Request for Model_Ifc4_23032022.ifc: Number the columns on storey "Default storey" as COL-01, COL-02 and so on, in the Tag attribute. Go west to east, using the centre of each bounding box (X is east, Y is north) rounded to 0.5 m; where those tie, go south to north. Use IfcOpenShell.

First a look at what the model holds.

```python
import ifcopenshell
import ifcopenshell.util.element
import ifcopenshell.util.placement

model = ifcopenshell.open("Model_Ifc4_23032022.ifc")
print(model.schema)
storey = next(s for s in model.by_type("IfcBuildingStorey") if s.Name == "Default storey")
columns = [e for e in ifcopenshell.util.element.get_decomposition(storey) if e.is_a("IfcColumn")]
for e in sorted(columns, key=lambda e: e.id()):
    origin = ifcopenshell.util.placement.get_local_placement(e.ObjectPlacement)[:3, 3]
    print(e.id(), e.Tag, e.Name, origin.round(2) + 0.0, sep=" | ")
```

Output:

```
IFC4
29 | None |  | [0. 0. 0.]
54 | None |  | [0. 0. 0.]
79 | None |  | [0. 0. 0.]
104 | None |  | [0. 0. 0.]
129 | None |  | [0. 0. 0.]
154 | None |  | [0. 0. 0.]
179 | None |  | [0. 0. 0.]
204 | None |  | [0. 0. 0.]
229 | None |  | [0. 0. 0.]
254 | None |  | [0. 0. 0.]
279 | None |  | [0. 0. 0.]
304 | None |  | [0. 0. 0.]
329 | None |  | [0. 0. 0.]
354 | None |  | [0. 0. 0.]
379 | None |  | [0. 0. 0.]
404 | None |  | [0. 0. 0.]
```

```python
import ifcopenshell
import ifcopenshell.geom
import ifcopenshell.util.element
import ifcopenshell.util.shape

model = ifcopenshell.open("Model_Ifc4_23032022.ifc")
settings = ifcopenshell.geom.settings()
settings.set("use-world-coords", True)


def centre(element):
    shape = ifcopenshell.geom.create_shape(settings, element)
    return ifcopenshell.util.shape.get_bbox_centroid(shape.geometry)


storey = next(s for s in model.by_type("IfcBuildingStorey") if s.Name == "Default storey")
columns = [e for e in ifcopenshell.util.element.get_decomposition(storey) if e.is_a("IfcColumn")]

# Insertion points can sit at a corner or the storey origin, so sort by the geometry (in metres).
centres = {e: centre(e) for e in columns}
columns.sort(key=lambda e: (round(centres[e][0] / 0.5), centres[e][1]))

for i, e in enumerate(columns, start=1):
    number = f"COL-{i:02d}"
    e.Tag = number
    print(e.id(), number)

model.write("Model_Ifc4_23032022_v2.ifc")
```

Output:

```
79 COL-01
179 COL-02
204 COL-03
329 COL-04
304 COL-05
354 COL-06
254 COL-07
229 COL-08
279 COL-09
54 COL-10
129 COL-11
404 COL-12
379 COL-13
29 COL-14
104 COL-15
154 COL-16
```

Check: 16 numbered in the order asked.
